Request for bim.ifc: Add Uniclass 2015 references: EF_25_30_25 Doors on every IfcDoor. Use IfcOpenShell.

First a look at what the model holds.

```python
import ifcopenshell

model = ifcopenshell.open("bim.ifc")
print(model.schema)
print("classifications:", [c.Name for c in model.by_type("IfcClassification")])
for ifc_class in ("IfcDoor", "IfcRoof", "IfcStair", "IfcWall", "IfcWindow"):
    print(ifc_class, len(model.by_type(ifc_class)))
```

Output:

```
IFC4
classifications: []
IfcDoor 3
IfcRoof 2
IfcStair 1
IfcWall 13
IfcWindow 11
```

```python
import ifcopenshell
import ifcopenshell.api.classification

model = ifcopenshell.open("bim.ifc")

system = ifcopenshell.api.classification.add_classification(model, classification="Uniclass 2015")

codes = {
    "IfcDoor": ("EF_25_30_25", "Doors"),
}
for ifc_class, (code, name) in codes.items():
    products = model.by_type(ifc_class)
    ifcopenshell.api.classification.add_reference(
        model, products=products, classification=system, identification=code, name=name
    )
    print(code, len(products))

model.write("bim_rev.ifc")
```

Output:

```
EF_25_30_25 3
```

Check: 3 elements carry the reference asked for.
